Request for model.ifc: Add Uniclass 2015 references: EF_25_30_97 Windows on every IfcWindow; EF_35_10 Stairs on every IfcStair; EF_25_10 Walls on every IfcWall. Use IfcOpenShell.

First a look at what the model holds.

```python
import ifcopenshell

model = ifcopenshell.open("model.ifc")
print(model.schema)
print("classifications:", [c.Name for c in model.by_type("IfcClassification")])
for ifc_class in ("IfcDoor", "IfcRoof", "IfcStair", "IfcWall", "IfcWindow"):
    print(ifc_class, len(model.by_type(ifc_class)))
```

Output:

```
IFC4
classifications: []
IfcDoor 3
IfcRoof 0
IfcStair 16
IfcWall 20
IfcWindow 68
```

```python
import ifcopenshell
import ifcopenshell.api.classification

model = ifcopenshell.open("model.ifc")

system = ifcopenshell.api.classification.add_classification(model, classification="Uniclass 2015")

codes = {
    "IfcWindow": ("EF_25_30_97", "Windows"),
    "IfcStair": ("EF_35_10", "Stairs"),
    "IfcWall": ("EF_25_10", "Walls"),
}
for ifc_class, (code, name) in codes.items():
    products = model.by_type(ifc_class)
    ifcopenshell.api.classification.add_reference(
        model, products=products, classification=system, identification=code, name=name
    )
    print(code, len(products))

model.write("model_rev.ifc")
```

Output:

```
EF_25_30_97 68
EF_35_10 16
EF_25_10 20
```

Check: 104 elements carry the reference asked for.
